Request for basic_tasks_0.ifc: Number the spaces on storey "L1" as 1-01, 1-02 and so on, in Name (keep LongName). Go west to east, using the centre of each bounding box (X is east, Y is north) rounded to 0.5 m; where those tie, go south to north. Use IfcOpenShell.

First a look at what the model holds.

```python
import ifcopenshell
import ifcopenshell.util.element
import ifcopenshell.util.placement

model = ifcopenshell.open("basic_tasks_0.ifc")
print(model.schema)
storey = next(s for s in model.by_type("IfcBuildingStorey") if s.Name == "L1")
spaces = [e for e in ifcopenshell.util.element.get_decomposition(storey) if e.is_a("IfcSpace")]
for e in sorted(spaces, key=lambda e: e.id()):
    origin = ifcopenshell.util.placement.get_local_placement(e.ObjectPlacement)[:3, 3]
    print(e.id(), e.Name, e.LongName, origin.round(2) + 0.0, sep=" | ")
```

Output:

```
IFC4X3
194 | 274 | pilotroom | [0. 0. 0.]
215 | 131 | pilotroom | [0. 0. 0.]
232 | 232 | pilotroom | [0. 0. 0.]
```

```python
import ifcopenshell
import ifcopenshell.geom
import ifcopenshell.util.element
import ifcopenshell.util.shape

model = ifcopenshell.open("basic_tasks_0.ifc")
settings = ifcopenshell.geom.settings()
settings.set("use-world-coords", True)


def centre(element):
    shape = ifcopenshell.geom.create_shape(settings, element)
    return ifcopenshell.util.shape.get_bbox_centroid(shape.geometry)


storey = next(s for s in model.by_type("IfcBuildingStorey") if s.Name == "L1")
spaces = [e for e in ifcopenshell.util.element.get_decomposition(storey) if e.is_a("IfcSpace")]

# Insertion points can sit at a corner or the storey origin, so sort by the geometry (in metres).
centres = {e: centre(e) for e in spaces}
spaces.sort(key=lambda e: (round(centres[e][0] / 0.5), centres[e][1]))

for i, e in enumerate(spaces, start=1):
    number = f"1-{i:02d}"
    e.Name = number
    print(e.id(), number)

model.write("basic_tasks_0-out.ifc")
```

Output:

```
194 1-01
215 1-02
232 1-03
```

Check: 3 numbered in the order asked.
